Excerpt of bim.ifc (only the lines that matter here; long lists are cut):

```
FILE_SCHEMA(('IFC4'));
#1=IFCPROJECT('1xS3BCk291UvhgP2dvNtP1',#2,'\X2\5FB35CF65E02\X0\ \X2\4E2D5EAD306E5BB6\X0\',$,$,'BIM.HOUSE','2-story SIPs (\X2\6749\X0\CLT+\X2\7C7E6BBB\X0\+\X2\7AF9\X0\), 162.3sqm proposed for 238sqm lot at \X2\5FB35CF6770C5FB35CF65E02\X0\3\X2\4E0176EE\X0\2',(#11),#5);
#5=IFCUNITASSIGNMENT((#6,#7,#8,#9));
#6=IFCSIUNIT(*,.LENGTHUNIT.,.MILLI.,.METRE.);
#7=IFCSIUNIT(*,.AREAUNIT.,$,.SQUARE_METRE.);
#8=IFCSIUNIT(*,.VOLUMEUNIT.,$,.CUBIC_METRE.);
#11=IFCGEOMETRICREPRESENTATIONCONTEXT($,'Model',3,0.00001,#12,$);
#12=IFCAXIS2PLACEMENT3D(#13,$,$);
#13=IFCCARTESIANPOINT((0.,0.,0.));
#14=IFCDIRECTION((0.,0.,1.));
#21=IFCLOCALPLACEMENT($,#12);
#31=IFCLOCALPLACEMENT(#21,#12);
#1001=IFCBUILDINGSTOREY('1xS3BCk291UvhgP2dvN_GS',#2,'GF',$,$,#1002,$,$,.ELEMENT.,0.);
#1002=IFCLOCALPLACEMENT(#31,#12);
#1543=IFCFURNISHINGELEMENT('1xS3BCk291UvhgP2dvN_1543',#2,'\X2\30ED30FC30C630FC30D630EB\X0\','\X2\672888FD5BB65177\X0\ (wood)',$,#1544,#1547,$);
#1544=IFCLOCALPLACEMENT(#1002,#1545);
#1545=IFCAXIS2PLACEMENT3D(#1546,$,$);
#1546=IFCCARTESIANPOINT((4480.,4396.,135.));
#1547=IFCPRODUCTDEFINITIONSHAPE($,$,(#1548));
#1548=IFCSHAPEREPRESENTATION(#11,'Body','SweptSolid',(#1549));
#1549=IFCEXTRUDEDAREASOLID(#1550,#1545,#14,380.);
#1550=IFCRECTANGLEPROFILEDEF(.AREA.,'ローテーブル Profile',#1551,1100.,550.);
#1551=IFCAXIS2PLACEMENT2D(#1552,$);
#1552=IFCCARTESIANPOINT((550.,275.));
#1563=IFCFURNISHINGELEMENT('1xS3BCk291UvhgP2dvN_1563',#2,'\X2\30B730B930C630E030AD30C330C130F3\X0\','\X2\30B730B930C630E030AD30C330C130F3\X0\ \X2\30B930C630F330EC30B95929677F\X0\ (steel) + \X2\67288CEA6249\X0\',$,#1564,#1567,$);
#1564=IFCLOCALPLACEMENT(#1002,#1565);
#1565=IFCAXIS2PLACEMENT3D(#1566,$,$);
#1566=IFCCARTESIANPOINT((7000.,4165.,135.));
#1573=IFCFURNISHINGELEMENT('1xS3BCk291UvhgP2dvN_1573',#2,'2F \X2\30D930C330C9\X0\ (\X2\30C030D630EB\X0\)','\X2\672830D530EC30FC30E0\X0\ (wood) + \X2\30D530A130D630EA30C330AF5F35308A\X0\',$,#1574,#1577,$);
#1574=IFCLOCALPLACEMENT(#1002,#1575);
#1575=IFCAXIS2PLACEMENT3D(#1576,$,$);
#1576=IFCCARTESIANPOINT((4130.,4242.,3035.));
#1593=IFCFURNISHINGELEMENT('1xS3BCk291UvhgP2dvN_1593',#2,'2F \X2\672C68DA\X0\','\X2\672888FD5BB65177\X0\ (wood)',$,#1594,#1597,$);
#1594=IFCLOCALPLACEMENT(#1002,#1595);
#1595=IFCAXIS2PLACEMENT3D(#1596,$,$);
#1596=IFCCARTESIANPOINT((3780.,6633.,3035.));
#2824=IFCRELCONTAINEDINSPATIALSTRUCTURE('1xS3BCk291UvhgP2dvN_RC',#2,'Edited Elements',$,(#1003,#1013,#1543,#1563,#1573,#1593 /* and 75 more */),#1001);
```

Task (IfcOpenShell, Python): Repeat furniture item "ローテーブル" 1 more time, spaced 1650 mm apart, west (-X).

```python
import numpy as np
import ifcopenshell
import ifcopenshell.api.geometry
import ifcopenshell.api.root
import ifcopenshell.util.element
import ifcopenshell.util.placement

model = ifcopenshell.open("bim.ifc")


def reuse_history(source, copy):
    """copy_class also copies each property set's owner history, people and application; keep the originals."""
    for rel in copy.IsDefinedBy:
        if rel.is_a("IfcRelDefinesByProperties") and (history := rel.RelatingPropertyDefinition.OwnerHistory):
            rel.RelatingPropertyDefinition.OwnerHistory = source.OwnerHistory
            ifcopenshell.util.element.remove_deep2(model, history)


source = model.by_guid("1xS3BCk291UvhgP2dvN_1543")
base = ifcopenshell.util.placement.get_local_placement(source.ObjectPlacement)
step = np.array([-1.0, 0.0, 0.0]) * 1650.0

for i in range(1, 2):
    copy = ifcopenshell.api.root.copy_class(model, product=source)
    copy.Representation = ifcopenshell.util.element.copy_deep(
        model, source.Representation, exclude=["IfcGeometricRepresentationContext", "IfcRepresentationMap"]
    )
    reuse_history(source, copy)
    matrix = base.copy()
    matrix[:3, 3] += i * step
    print("added at", matrix[:3, 3].round(3) + 0.0)
    ifcopenshell.api.geometry.edit_object_placement(model, product=copy, matrix=matrix, is_si=False)

model.write("bim_rev.ifc")
```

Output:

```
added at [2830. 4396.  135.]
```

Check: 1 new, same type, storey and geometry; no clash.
